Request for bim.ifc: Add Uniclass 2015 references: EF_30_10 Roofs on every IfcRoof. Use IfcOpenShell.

First a look at what the model holds.

```python
import ifcopenshell

model = ifcopenshell.open("bim.ifc")
print(model.schema)
print("classifications:", [c.Name for c in model.by_type("IfcClassification")])
for ifc_class in ("IfcDoor", "IfcRoof", "IfcStair", "IfcWall", "IfcWindow"):
    print(ifc_class, len(model.by_type(ifc_class)))
```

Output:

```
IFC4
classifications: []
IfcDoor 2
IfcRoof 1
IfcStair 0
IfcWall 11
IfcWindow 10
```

```python
import ifcopenshell
import ifcopenshell.api.classification

model = ifcopenshell.open("bim.ifc")

system = ifcopenshell.api.classification.add_classification(model, classification="Uniclass 2015")

codes = {
    "IfcRoof": ("EF_30_10", "Roofs"),
}
for ifc_class, (code, name) in codes.items():
    products = model.by_type(ifc_class)
    ifcopenshell.api.classification.add_reference(
        model, products=products, classification=system, identification=code, name=name
    )
    print(code, len(products))

model.write("bim_v2.ifc")
```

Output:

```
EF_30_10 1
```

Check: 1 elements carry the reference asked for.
